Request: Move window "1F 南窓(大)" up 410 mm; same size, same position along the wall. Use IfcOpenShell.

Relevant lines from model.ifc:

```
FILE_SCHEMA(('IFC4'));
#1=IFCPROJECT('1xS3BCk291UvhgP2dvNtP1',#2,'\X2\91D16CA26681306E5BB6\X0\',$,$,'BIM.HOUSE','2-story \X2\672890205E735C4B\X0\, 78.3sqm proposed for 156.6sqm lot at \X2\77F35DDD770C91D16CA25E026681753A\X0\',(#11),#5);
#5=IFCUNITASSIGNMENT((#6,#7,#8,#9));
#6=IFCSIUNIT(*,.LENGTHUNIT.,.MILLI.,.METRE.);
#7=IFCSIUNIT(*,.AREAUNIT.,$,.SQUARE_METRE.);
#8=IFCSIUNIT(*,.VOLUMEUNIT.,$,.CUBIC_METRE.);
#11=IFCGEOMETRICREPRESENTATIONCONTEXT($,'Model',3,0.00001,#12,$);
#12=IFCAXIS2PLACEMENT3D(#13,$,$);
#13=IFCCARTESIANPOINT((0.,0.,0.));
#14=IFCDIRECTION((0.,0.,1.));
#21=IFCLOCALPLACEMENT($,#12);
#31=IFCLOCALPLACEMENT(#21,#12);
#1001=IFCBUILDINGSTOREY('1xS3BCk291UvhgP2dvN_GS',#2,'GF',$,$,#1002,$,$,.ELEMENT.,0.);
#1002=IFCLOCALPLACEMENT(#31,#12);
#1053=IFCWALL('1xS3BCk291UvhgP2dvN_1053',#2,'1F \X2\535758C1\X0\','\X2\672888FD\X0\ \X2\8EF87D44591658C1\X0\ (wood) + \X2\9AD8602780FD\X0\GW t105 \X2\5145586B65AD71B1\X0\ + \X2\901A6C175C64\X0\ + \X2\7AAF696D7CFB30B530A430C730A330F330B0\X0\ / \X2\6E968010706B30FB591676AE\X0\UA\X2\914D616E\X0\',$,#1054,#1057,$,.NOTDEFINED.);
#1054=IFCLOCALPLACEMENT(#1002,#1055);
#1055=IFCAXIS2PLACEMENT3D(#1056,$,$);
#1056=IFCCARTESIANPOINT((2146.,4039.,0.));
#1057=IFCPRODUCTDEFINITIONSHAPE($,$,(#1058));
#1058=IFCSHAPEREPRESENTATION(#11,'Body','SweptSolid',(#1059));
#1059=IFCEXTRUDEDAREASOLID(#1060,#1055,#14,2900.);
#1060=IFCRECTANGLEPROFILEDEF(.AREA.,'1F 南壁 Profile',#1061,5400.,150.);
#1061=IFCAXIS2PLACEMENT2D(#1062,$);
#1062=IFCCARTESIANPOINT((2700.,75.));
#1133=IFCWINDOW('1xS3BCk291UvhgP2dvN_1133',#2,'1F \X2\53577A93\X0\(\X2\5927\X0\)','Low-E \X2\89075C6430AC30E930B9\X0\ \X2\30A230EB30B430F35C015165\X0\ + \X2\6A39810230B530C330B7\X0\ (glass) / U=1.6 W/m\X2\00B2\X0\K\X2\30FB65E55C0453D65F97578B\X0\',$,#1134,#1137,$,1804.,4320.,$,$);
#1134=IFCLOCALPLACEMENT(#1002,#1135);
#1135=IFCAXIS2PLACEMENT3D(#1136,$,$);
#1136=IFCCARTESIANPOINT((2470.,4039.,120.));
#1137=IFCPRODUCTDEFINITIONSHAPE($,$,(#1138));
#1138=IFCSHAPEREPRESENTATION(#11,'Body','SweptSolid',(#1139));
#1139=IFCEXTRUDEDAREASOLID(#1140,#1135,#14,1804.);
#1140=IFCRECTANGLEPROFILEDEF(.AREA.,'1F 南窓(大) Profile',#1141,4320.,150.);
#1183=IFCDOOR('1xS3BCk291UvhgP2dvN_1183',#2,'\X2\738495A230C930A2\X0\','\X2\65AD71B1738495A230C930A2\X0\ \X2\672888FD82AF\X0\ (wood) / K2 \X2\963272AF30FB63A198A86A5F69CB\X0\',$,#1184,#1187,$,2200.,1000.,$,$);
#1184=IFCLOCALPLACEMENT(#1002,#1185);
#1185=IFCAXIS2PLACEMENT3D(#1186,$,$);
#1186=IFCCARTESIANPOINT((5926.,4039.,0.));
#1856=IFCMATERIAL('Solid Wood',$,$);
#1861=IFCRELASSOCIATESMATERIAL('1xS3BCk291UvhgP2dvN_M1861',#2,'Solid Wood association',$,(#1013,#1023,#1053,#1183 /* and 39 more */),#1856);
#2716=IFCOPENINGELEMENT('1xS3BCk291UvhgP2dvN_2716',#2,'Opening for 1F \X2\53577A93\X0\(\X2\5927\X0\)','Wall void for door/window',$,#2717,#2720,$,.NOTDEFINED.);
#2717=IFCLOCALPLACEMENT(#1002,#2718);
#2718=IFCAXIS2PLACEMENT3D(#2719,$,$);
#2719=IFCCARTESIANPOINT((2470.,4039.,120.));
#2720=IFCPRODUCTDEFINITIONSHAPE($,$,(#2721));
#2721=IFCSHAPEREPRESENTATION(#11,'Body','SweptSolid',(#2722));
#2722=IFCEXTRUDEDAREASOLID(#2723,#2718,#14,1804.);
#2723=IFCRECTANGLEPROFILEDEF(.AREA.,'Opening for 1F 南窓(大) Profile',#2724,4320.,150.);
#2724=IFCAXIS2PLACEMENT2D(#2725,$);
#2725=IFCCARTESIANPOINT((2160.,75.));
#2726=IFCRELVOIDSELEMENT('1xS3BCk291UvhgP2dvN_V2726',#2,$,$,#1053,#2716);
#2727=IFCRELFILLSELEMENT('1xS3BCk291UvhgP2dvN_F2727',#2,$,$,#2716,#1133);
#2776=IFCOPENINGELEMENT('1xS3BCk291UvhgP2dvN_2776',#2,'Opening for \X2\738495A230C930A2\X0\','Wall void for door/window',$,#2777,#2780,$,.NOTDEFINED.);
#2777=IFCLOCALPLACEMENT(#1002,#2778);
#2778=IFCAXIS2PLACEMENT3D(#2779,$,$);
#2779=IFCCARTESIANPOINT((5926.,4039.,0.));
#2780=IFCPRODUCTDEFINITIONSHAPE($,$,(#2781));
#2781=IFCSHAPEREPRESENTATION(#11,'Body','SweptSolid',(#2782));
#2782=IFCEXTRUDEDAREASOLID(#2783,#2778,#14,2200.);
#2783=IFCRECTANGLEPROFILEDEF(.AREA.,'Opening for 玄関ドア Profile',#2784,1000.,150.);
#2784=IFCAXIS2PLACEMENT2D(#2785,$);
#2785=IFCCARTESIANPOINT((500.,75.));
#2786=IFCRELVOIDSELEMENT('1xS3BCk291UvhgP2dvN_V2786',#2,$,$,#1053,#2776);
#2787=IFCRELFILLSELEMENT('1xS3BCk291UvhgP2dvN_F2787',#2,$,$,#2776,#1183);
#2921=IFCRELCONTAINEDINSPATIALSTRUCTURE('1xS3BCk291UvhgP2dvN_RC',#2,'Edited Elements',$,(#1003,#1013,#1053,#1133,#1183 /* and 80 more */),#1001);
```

```python
import numpy as np
import ifcopenshell
import ifcopenshell.api.geometry
import ifcopenshell.util.placement
import ifcopenshell.util.unit

model = ifcopenshell.open("model.ifc")
unit_scale = ifcopenshell.util.unit.calculate_unit_scale(model)

window = model.by_guid("1xS3BCk291UvhgP2dvN_1133")
opening = window.FillsVoids[0].RelatingOpeningElement
dz = 0.41 / unit_scale

shift = np.array([0.0, 0.0, dz])
# The window is not placed relative to its opening, so move both.
for product in (opening, window):
    matrix = ifcopenshell.util.placement.get_local_placement(product.ObjectPlacement)
    matrix[:3, 3] += shift
    ifcopenshell.api.geometry.edit_object_placement(model, product=product, matrix=matrix, is_si=False)

print(f"moved by {dz * unit_scale:+.3f} m")

model.write("model-out.ifc")
```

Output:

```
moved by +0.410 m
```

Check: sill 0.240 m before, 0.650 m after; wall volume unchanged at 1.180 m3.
